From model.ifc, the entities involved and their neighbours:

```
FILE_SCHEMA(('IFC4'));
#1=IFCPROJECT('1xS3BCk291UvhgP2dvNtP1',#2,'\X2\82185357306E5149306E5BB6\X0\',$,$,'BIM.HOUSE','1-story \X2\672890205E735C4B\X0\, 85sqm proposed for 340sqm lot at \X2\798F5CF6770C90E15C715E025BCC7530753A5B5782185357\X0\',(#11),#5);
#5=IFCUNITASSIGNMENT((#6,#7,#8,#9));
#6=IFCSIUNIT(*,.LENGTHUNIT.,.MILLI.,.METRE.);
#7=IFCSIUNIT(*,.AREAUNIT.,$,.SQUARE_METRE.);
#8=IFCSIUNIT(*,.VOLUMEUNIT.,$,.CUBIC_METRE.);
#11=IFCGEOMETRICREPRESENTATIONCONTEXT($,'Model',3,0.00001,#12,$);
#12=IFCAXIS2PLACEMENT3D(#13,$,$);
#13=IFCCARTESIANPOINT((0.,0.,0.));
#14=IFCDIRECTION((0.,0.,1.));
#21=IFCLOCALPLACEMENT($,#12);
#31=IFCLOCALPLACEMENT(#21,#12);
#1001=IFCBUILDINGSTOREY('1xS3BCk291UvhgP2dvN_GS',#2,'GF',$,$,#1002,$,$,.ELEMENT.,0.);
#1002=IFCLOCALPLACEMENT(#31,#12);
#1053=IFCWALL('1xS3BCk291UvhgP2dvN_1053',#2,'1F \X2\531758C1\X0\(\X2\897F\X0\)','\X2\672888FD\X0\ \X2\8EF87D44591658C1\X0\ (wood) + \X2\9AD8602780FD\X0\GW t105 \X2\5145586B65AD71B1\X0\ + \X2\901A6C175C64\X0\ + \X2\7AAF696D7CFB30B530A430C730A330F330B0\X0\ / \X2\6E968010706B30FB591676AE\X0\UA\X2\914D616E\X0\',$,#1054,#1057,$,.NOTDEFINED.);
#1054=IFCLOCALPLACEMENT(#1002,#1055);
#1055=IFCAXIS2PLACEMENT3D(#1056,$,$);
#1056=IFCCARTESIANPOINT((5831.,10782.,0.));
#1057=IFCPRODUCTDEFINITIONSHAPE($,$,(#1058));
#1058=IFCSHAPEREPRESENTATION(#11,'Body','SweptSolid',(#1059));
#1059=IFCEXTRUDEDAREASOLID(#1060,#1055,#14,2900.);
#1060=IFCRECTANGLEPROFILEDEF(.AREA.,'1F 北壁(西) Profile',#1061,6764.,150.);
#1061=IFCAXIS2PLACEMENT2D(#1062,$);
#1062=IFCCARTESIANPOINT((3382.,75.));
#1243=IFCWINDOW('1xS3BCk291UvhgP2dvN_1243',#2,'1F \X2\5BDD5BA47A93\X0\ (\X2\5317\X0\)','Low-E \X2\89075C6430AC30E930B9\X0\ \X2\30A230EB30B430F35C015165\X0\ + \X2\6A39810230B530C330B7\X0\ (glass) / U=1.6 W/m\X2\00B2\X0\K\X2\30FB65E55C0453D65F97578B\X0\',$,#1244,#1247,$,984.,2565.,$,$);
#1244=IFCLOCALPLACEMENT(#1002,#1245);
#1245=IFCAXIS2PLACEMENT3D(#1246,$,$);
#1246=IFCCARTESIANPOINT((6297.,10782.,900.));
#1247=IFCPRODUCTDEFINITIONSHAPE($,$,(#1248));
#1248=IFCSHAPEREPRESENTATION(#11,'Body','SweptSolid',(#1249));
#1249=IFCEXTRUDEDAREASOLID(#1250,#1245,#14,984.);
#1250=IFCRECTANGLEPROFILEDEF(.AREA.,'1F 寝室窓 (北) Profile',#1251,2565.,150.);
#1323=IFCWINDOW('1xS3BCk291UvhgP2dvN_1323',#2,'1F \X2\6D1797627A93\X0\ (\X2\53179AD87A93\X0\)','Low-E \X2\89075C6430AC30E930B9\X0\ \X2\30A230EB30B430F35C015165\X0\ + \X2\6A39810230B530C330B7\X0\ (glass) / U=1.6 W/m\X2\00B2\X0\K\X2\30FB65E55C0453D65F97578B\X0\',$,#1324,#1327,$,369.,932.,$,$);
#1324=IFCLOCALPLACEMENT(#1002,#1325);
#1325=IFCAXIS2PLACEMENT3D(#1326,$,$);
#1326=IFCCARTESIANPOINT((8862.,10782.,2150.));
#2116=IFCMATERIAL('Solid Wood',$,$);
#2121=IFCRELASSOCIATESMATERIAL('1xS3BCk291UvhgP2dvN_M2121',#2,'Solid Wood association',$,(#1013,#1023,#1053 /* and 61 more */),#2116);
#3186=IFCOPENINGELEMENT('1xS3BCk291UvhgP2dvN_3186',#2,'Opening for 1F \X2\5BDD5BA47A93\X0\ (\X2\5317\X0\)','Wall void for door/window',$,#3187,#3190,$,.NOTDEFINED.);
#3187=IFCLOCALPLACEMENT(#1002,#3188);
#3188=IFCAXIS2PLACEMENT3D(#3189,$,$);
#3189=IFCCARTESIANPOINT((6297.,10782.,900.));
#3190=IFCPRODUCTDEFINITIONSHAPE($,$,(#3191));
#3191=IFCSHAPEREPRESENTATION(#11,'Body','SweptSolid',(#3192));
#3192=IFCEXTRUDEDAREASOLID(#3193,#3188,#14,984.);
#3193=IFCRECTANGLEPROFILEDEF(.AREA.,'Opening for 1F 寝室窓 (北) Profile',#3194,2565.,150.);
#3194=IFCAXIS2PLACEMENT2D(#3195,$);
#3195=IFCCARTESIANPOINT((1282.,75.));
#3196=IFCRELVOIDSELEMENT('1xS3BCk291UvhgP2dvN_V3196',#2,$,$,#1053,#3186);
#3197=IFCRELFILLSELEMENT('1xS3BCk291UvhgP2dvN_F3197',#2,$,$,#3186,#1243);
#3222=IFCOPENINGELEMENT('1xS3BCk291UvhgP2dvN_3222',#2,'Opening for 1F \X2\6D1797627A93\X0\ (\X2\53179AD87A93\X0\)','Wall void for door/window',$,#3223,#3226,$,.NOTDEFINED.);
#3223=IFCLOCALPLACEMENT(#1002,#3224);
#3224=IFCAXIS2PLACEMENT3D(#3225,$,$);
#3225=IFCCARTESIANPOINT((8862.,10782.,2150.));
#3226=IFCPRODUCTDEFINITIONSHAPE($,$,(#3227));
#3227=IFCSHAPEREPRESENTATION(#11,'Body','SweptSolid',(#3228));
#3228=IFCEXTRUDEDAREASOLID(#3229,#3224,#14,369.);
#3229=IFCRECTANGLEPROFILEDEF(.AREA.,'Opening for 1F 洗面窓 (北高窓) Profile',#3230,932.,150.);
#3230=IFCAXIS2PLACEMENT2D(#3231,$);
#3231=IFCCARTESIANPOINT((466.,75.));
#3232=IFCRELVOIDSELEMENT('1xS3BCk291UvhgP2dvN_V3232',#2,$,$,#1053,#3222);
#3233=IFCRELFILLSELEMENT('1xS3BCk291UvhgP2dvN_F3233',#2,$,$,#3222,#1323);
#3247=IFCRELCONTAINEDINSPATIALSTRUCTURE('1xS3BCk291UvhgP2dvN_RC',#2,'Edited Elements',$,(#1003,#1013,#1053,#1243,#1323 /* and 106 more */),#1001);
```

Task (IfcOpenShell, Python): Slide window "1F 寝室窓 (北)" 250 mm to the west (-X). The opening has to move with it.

```python
import ifcopenshell
import ifcopenshell.api.geometry
import ifcopenshell.util.placement
import ifcopenshell.util.unit

model = ifcopenshell.open("model.ifc")
unit_scale = ifcopenshell.util.unit.calculate_unit_scale(model)

window = model.by_guid("1xS3BCk291UvhgP2dvN_1243")
opening = window.FillsVoids[0].RelatingOpeningElement
wall = opening.VoidsElements[0].RelatingBuildingElement

wall_matrix = ifcopenshell.util.placement.get_local_placement(wall.ObjectPlacement)
shift = wall_matrix[:3, 0] * -0.25 / unit_scale
before = ifcopenshell.util.placement.get_local_placement(window.ObjectPlacement)[:3, 3].copy()

# The window is not placed relative to its opening, so move both.
for product in (opening, window):
    matrix = ifcopenshell.util.placement.get_local_placement(product.ObjectPlacement)
    matrix[:3, 3] += shift
    ifcopenshell.api.geometry.edit_object_placement(model, product=product, matrix=matrix, is_si=False)

after = ifcopenshell.util.placement.get_local_placement(window.ObjectPlacement)[:3, 3]
print("window moved by", (after - before).round(3) + 0.0)

model.write("model-out.ifc")
```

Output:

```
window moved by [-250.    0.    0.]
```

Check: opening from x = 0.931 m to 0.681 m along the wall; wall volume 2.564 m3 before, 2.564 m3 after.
